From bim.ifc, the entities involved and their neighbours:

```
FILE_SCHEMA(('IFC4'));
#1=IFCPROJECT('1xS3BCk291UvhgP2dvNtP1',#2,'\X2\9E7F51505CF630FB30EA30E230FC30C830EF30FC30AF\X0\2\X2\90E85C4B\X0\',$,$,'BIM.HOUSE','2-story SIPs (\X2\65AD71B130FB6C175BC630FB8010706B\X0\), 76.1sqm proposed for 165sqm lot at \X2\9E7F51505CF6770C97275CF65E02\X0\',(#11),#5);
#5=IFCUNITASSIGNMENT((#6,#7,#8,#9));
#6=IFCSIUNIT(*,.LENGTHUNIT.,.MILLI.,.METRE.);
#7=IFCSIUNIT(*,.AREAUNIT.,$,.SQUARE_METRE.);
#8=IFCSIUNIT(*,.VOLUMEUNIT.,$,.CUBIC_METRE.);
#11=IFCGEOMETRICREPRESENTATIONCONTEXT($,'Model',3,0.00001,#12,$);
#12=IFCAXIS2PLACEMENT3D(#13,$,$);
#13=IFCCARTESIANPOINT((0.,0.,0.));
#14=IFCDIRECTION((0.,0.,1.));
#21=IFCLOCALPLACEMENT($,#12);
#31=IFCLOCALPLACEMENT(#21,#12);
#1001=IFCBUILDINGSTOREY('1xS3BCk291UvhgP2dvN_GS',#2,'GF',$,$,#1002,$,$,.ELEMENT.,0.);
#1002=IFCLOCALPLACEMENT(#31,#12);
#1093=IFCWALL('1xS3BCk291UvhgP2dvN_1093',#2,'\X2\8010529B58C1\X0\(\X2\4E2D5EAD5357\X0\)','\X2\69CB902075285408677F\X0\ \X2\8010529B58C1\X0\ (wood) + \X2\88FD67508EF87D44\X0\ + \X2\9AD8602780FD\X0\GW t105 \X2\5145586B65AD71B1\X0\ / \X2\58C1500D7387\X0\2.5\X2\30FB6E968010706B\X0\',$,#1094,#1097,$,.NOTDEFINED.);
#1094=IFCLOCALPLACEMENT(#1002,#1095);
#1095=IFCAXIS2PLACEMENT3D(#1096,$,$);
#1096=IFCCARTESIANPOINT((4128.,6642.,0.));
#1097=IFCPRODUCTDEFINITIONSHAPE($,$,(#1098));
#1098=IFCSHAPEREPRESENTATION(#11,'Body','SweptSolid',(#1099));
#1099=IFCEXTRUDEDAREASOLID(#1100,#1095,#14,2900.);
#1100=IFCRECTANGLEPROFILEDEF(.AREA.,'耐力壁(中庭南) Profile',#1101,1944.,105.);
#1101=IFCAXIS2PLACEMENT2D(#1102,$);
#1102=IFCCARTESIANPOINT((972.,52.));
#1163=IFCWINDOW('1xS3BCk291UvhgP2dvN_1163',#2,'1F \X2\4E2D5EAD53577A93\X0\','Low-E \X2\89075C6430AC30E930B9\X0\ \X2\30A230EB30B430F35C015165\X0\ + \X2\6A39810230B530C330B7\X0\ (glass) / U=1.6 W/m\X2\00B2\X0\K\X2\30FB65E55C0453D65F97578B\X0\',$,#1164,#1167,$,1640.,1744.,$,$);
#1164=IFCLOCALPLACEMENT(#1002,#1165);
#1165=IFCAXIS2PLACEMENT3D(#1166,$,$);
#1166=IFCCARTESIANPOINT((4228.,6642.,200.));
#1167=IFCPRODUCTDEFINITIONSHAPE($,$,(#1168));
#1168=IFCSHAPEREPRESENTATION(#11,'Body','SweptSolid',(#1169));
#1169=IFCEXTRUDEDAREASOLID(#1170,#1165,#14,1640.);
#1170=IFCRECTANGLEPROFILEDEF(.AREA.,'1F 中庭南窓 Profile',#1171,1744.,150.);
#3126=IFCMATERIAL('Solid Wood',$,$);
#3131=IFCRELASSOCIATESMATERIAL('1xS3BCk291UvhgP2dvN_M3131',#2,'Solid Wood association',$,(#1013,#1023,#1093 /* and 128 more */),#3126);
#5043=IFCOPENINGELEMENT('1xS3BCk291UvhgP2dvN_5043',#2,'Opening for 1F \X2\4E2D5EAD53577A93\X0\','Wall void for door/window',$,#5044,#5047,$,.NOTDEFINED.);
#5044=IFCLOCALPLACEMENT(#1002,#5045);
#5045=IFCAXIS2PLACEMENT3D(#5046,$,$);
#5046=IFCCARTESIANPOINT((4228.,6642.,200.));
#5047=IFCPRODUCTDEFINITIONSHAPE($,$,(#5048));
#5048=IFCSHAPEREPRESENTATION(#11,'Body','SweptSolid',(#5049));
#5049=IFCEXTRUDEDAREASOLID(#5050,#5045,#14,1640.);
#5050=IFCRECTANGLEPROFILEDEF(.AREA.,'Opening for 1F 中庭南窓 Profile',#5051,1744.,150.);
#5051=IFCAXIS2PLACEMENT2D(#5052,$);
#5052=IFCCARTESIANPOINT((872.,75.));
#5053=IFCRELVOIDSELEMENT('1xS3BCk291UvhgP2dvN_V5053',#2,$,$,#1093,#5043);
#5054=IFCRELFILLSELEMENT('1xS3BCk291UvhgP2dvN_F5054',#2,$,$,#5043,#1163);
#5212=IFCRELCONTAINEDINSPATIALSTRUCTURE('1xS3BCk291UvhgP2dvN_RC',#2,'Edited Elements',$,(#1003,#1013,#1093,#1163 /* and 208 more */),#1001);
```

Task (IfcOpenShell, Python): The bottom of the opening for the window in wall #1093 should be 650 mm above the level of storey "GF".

```python
import numpy as np
import ifcopenshell
import ifcopenshell.api.geometry
import ifcopenshell.geom
import ifcopenshell.util.element
import ifcopenshell.util.placement
import ifcopenshell.util.shape
import ifcopenshell.util.unit

model = ifcopenshell.open("bim.ifc")
unit_scale = ifcopenshell.util.unit.calculate_unit_scale(model)

window = model.by_guid("1xS3BCk291UvhgP2dvN_1163")
opening = window.FillsVoids[0].RelatingOpeningElement
storey = ifcopenshell.util.element.get_container(window, ifc_class="IfcBuildingStorey")
level = ifcopenshell.util.placement.get_local_placement(storey.ObjectPlacement)[2, 3]

# The opening's origin need not be at the sill, so measure its lowest point.
shape = ifcopenshell.geom.create_shape(ifcopenshell.geom.settings(), opening)
bottom = ifcopenshell.util.shape.get_shape_bottom_elevation(shape, shape.geometry) / unit_scale
dz = level + 0.65 / unit_scale - bottom

shift = np.array([0.0, 0.0, dz])
# The window is not placed relative to its opening, so move both.
for product in (opening, window):
    matrix = ifcopenshell.util.placement.get_local_placement(product.ObjectPlacement)
    matrix[:3, 3] += shift
    ifcopenshell.api.geometry.edit_object_placement(model, product=product, matrix=matrix, is_si=False)

print(f"moved by {dz * unit_scale:+.3f} m")

model.write("bim-out.ifc")
```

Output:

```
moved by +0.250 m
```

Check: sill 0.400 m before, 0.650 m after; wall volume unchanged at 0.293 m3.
